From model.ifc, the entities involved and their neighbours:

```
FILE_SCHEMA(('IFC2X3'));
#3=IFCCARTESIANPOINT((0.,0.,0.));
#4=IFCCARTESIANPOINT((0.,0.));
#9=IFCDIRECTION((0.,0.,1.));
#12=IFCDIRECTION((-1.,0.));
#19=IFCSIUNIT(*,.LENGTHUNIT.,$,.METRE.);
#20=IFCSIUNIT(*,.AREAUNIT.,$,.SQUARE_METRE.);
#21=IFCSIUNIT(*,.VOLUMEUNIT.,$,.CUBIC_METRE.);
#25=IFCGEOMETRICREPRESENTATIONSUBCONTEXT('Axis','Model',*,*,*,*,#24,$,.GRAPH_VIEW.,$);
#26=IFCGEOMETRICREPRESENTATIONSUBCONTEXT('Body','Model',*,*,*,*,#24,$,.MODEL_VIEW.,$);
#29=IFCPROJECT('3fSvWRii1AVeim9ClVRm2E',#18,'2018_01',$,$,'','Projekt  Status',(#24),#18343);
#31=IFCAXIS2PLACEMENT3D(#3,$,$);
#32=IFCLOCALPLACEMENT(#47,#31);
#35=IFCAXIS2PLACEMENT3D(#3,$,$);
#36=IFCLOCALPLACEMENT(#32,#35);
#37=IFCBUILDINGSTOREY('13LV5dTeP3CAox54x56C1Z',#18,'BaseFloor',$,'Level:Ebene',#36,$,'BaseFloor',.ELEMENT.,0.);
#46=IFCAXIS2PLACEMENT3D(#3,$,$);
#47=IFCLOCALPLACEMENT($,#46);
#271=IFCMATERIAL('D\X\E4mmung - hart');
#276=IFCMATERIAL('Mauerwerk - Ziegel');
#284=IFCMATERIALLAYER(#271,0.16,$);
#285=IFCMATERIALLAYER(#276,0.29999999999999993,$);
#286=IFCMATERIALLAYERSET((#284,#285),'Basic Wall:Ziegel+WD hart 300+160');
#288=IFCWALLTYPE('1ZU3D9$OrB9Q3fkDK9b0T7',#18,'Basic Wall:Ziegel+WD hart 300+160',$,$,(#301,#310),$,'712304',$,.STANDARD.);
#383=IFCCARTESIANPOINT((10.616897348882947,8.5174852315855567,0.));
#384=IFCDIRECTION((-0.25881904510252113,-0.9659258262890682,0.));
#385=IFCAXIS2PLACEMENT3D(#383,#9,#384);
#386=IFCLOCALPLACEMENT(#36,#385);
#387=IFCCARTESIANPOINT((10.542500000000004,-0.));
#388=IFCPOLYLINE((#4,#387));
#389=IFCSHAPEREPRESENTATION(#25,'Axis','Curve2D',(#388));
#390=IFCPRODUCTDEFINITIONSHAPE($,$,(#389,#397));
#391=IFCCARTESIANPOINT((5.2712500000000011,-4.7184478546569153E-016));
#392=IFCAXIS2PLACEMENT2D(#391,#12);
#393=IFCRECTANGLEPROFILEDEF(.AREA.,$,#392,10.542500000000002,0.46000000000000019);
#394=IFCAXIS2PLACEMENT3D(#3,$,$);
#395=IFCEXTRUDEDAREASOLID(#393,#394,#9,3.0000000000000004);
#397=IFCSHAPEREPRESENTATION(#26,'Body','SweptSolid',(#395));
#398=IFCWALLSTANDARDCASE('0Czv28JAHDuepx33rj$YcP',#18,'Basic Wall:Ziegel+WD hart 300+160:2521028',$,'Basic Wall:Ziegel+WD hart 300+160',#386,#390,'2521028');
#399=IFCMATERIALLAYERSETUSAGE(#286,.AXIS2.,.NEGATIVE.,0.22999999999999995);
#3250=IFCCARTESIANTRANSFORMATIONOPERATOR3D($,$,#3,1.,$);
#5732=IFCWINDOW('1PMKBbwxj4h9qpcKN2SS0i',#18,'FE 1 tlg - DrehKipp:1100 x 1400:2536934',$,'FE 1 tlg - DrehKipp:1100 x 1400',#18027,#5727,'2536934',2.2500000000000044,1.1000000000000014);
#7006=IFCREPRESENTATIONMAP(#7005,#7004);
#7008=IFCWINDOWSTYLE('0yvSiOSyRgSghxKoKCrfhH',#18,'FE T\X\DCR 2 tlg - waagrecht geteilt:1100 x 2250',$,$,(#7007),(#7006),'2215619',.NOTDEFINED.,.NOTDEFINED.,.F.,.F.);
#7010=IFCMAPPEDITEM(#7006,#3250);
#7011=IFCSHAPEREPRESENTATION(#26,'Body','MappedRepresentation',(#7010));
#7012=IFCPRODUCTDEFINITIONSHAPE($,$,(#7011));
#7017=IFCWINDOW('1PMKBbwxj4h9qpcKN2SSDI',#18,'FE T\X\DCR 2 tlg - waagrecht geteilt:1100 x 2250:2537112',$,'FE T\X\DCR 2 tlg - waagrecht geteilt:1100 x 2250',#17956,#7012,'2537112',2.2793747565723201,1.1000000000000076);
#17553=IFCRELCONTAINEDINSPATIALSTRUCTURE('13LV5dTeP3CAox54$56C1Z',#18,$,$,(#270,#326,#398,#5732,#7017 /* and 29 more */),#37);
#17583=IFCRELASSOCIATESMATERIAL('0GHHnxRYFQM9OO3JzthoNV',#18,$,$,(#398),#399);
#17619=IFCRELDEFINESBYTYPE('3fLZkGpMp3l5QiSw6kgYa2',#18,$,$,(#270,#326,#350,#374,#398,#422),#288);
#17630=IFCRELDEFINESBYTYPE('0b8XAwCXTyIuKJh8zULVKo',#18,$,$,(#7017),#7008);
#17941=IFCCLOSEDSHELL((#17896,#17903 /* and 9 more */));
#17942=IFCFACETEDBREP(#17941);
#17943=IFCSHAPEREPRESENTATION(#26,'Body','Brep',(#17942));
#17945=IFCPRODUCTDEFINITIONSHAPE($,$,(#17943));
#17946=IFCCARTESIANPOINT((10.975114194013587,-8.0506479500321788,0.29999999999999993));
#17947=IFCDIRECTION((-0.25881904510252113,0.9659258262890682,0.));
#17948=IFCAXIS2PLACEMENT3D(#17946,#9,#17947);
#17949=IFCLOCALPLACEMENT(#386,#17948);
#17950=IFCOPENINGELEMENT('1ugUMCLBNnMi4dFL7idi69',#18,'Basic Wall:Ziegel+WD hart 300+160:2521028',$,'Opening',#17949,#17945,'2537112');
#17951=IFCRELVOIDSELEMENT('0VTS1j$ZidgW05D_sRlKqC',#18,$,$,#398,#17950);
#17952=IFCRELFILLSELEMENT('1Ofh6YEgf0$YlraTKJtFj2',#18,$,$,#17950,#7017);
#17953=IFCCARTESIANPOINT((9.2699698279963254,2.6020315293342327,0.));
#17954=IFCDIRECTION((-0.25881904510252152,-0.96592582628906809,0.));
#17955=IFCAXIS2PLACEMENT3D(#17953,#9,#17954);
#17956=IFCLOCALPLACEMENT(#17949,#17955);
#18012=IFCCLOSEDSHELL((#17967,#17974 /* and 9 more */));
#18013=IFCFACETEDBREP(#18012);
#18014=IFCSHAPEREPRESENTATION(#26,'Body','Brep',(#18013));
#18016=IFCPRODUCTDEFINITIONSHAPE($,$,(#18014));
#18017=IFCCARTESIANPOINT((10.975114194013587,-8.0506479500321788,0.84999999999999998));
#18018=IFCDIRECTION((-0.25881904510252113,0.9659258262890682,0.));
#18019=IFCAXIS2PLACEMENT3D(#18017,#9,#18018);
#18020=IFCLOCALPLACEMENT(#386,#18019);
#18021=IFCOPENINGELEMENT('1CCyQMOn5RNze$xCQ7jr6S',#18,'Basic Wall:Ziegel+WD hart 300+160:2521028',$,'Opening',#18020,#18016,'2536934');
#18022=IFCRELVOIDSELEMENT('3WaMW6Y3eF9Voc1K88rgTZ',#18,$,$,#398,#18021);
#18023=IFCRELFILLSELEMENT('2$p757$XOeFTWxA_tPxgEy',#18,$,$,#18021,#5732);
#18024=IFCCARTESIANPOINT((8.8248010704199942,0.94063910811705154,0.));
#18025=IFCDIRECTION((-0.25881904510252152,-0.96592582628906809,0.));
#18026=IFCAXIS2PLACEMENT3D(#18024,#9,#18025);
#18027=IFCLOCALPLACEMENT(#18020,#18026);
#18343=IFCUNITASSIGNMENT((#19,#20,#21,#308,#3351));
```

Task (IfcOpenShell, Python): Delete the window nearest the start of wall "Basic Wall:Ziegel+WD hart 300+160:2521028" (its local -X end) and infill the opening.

```python
import ifcopenshell
import ifcopenshell.api.feature
import ifcopenshell.api.root
import ifcopenshell.geom
import ifcopenshell.util.shape

model = ifcopenshell.open("model.ifc")
settings = ifcopenshell.geom.settings()


def volume(element):
    """Net volume in cubic metres, openings subtracted."""
    shape = ifcopenshell.geom.create_shape(settings, element)
    return ifcopenshell.util.shape.get_volume(shape.geometry)


window = model.by_guid("1PMKBbwxj4h9qpcKN2SSDI")
opening = window.FillsVoids[0].RelatingOpeningElement
wall = opening.VoidsElements[0].RelatingBuildingElement
before = volume(wall)

ifcopenshell.api.root.remove_product(model, product=window)
ifcopenshell.api.feature.remove_feature(model, feature=opening)

after = volume(wall)

print(f"wall volume {before:.3f} -> {after:.3f} m3")

model.write("model-out.ifc")
```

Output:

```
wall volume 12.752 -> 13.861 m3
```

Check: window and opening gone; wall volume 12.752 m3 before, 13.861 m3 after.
